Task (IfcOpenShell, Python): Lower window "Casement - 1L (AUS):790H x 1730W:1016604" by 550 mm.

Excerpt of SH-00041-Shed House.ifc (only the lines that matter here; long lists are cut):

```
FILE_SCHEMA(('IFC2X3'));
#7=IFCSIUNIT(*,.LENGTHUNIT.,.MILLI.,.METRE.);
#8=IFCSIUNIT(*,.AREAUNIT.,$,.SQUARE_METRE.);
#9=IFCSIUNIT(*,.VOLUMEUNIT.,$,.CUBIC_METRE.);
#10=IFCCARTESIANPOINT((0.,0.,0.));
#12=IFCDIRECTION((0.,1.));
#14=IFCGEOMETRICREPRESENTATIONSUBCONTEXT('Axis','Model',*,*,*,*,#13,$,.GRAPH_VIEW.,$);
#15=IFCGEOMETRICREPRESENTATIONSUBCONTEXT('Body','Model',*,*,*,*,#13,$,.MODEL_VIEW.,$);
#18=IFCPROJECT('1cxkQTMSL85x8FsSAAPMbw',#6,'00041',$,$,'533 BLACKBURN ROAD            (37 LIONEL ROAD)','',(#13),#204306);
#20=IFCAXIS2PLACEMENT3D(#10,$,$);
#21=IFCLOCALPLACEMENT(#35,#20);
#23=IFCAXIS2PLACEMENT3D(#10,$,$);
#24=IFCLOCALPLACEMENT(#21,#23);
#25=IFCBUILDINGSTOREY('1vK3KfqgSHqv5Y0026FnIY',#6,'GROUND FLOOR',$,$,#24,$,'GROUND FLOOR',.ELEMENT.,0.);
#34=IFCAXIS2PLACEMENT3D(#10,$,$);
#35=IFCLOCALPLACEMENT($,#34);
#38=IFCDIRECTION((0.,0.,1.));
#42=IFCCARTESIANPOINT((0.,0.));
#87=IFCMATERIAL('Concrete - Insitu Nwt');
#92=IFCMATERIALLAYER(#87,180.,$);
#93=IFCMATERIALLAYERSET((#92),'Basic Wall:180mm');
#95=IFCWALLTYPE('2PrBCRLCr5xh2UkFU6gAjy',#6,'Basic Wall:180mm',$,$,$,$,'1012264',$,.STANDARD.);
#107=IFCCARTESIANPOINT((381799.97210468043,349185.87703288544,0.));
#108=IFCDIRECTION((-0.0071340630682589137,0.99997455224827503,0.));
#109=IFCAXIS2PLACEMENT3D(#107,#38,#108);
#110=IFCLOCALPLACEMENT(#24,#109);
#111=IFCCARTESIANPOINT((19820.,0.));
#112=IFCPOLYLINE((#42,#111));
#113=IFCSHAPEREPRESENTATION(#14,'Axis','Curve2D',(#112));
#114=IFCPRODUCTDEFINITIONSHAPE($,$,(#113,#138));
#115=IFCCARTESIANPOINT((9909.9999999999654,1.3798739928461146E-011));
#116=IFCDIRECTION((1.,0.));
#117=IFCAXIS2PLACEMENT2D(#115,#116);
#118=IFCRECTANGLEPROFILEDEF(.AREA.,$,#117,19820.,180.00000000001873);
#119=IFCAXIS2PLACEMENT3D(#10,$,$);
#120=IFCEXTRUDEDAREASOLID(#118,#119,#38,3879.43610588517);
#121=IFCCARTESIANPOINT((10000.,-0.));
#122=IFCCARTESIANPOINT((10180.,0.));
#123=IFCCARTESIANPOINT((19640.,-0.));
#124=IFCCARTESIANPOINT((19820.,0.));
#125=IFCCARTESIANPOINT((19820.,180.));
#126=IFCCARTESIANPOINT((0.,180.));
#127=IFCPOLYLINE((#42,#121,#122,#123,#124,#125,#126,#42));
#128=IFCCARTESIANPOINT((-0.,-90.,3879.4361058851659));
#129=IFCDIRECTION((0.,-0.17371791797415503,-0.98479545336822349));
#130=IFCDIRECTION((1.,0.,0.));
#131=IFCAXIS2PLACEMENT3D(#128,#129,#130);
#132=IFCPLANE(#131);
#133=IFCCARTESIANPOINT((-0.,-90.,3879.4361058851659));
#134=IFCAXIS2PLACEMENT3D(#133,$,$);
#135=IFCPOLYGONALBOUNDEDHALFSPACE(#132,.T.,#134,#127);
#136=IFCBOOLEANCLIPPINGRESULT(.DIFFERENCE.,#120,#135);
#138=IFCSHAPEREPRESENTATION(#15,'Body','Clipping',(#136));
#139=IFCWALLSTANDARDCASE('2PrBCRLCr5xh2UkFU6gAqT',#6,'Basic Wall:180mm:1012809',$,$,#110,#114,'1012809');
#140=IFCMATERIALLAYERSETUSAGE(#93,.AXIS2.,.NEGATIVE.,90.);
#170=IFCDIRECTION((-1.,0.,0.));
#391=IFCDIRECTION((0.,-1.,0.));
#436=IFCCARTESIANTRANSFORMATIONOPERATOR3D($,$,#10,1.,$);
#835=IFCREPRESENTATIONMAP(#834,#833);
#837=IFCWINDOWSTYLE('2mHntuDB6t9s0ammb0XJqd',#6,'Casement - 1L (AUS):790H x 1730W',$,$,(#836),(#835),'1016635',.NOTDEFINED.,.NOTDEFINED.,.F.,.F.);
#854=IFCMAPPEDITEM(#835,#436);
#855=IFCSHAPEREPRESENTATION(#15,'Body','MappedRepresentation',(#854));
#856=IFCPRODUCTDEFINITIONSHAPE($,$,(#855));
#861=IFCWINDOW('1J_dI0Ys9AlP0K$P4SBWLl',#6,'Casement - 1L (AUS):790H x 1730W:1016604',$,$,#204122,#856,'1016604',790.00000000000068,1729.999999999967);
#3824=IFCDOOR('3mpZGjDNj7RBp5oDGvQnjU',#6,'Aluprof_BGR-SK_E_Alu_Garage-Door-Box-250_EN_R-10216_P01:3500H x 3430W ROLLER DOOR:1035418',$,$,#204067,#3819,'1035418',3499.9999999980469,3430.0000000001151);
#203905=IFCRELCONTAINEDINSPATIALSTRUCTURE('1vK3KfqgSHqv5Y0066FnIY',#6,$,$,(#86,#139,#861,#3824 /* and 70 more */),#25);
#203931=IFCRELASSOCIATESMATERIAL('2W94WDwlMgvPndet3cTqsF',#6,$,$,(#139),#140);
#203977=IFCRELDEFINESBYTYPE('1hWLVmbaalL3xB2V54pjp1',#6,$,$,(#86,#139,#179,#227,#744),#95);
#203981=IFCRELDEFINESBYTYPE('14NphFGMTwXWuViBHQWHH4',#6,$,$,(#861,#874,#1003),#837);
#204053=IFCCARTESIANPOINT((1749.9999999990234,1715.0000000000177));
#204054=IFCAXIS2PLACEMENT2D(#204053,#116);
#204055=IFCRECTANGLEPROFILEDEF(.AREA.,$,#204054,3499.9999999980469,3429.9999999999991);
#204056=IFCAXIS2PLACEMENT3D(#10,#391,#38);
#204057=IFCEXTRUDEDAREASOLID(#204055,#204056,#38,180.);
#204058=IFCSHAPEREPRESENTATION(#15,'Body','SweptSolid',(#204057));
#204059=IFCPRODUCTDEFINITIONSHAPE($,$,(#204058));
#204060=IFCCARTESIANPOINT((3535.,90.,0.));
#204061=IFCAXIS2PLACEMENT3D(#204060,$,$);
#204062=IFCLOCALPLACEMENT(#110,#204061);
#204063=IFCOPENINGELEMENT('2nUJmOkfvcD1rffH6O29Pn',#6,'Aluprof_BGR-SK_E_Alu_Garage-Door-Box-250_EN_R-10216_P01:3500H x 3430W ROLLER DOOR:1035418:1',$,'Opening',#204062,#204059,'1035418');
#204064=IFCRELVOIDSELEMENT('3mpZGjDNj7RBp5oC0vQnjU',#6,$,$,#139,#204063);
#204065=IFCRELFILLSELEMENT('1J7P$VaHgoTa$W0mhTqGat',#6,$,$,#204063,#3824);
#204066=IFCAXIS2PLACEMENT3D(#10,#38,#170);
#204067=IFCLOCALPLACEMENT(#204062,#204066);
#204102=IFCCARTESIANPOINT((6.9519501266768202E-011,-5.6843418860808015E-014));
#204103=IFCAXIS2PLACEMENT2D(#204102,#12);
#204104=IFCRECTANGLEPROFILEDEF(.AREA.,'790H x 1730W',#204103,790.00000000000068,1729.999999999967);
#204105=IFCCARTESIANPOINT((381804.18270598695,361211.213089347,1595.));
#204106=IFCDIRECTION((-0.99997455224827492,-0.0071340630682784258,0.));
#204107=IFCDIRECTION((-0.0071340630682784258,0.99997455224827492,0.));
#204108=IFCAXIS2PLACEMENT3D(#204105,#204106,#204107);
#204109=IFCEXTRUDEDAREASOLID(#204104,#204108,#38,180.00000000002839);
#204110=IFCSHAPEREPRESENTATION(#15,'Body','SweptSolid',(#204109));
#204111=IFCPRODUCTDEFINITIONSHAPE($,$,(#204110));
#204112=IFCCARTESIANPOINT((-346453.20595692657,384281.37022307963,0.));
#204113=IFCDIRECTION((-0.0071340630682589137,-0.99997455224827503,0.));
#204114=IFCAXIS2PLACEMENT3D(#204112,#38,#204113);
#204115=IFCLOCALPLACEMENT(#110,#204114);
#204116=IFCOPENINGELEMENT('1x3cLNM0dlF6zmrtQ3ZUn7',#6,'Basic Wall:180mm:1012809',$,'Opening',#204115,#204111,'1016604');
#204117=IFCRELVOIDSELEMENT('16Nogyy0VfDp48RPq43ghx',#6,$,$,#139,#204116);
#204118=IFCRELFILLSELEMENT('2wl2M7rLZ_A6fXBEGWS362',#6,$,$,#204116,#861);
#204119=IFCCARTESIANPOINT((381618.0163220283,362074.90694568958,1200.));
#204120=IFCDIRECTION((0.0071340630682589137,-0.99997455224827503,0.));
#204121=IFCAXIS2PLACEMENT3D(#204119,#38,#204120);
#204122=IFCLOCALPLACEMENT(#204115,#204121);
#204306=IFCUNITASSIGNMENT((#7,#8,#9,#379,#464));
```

```python
import numpy as np
import ifcopenshell
import ifcopenshell.api.geometry
import ifcopenshell.util.placement
import ifcopenshell.util.unit

model = ifcopenshell.open("SH-00041-Shed House.ifc")
unit_scale = ifcopenshell.util.unit.calculate_unit_scale(model)

window = model.by_guid("1J_dI0Ys9AlP0K$P4SBWLl")
opening = window.FillsVoids[0].RelatingOpeningElement
dz = -0.55 / unit_scale

shift = np.array([0.0, 0.0, dz])
# The window is placed relative to its opening, so it follows when the opening moves.
matrix = ifcopenshell.util.placement.get_local_placement(opening.ObjectPlacement)
matrix[:3, 3] += shift
ifcopenshell.api.geometry.edit_object_placement(
    model, product=opening, matrix=matrix, is_si=False, should_transform_children=True
)

print(f"moved by {dz * unit_scale:+.3f} m")

model.write("SH-00041-Shed House_edited.ifc")
```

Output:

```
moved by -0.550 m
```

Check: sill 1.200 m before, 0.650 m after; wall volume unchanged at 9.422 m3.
